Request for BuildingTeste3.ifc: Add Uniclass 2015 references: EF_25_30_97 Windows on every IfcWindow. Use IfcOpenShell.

First a look at what the model holds.

```python
import ifcopenshell

model = ifcopenshell.open("BuildingTeste3.ifc")
print(model.schema)
print("classifications:", [c.Name for c in model.by_type("IfcClassification")])
for ifc_class in ("IfcDoor", "IfcRoof", "IfcStair", "IfcWall", "IfcWindow"):
    print(ifc_class, len(model.by_type(ifc_class)))
```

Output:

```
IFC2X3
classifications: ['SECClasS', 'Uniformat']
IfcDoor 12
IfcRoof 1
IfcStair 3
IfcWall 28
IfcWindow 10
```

```python
import ifcopenshell
import ifcopenshell.api.classification

model = ifcopenshell.open("BuildingTeste3.ifc")

# IFC2X3 requires Source and Edition and has no link from the project to the system.
system = model.create_entity("IfcClassification", Source="NBS", Edition="2015", Name="Uniclass 2015")

codes = {
    "IfcWindow": ("EF_25_30_97", "Windows"),
}
for ifc_class, (code, name) in codes.items():
    products = model.by_type(ifc_class)
    ifcopenshell.api.classification.add_reference(
        model, products=products, classification=system, identification=code, name=name
    )
    print(code, len(products))

model.write("BuildingTeste3-out.ifc")
```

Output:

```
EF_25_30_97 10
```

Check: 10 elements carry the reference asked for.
